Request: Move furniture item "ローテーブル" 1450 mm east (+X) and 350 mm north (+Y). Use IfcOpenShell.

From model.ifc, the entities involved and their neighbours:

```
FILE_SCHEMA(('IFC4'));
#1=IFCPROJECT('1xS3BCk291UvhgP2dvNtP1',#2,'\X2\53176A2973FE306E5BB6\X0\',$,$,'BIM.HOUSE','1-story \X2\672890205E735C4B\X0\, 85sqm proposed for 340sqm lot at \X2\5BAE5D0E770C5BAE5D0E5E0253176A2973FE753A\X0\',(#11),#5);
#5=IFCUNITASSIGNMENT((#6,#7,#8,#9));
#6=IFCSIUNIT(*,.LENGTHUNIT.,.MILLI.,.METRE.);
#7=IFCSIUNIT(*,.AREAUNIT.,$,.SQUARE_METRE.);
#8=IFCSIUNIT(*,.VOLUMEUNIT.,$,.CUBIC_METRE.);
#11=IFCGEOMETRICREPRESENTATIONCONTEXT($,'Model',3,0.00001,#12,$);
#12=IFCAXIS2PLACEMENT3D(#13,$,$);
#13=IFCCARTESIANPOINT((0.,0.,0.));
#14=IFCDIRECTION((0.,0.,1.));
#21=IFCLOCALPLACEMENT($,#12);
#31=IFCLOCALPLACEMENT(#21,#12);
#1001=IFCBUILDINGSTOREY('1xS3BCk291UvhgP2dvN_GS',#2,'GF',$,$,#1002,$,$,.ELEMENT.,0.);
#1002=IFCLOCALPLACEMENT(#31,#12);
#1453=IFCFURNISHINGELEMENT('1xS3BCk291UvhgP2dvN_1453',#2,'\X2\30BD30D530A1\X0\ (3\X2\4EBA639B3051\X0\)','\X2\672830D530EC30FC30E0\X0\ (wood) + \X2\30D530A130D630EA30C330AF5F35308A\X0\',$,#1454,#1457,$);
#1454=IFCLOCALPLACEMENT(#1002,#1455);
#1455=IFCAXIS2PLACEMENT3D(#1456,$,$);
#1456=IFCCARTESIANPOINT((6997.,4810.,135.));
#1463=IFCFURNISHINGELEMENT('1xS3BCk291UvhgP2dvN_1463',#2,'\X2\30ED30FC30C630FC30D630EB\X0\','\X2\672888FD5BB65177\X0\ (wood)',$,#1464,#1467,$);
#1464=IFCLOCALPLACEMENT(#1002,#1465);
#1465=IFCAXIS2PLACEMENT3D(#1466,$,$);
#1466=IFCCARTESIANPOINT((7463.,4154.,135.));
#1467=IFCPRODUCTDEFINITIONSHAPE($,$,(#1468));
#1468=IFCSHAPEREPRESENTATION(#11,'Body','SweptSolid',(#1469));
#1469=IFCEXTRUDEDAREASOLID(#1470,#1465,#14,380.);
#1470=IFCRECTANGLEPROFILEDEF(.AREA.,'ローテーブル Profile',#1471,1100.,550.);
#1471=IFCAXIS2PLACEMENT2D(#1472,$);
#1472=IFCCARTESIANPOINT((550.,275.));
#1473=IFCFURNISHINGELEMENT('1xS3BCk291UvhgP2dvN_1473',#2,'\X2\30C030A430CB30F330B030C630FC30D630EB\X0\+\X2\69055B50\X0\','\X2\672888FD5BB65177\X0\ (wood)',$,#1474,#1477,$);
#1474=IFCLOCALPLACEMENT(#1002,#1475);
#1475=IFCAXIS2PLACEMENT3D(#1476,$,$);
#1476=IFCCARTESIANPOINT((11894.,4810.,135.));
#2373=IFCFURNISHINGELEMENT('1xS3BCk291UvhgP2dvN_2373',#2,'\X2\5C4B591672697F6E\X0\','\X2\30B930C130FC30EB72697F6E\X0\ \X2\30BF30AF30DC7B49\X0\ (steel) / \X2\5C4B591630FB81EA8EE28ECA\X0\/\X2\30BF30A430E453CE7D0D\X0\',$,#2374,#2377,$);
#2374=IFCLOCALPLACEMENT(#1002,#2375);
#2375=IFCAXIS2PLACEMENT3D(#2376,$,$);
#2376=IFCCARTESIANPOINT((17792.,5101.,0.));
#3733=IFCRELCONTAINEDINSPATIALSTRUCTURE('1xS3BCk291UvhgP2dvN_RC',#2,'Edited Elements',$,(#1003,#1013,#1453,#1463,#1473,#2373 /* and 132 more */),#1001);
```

```python
import ifcopenshell
import ifcopenshell.api.geometry
import ifcopenshell.util.placement
import ifcopenshell.util.unit

model = ifcopenshell.open("model.ifc")
unit_scale = ifcopenshell.util.unit.calculate_unit_scale(model)

item = model.by_guid("1xS3BCk291UvhgP2dvN_1463")
matrix = ifcopenshell.util.placement.get_local_placement(item.ObjectPlacement)
matrix[0, 3] += 1.45 / unit_scale
matrix[1, 3] += 0.35 / unit_scale
ifcopenshell.api.geometry.edit_object_placement(model, product=item, matrix=matrix, is_si=False)

print(ifcopenshell.util.placement.get_local_placement(item.ObjectPlacement).round(3) + 0.0)

model.write("model_updated.ifc")
```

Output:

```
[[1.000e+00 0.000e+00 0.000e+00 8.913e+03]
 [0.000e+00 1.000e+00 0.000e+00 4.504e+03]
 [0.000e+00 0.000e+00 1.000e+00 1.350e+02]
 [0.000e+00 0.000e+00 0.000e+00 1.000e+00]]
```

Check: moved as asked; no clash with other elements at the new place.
